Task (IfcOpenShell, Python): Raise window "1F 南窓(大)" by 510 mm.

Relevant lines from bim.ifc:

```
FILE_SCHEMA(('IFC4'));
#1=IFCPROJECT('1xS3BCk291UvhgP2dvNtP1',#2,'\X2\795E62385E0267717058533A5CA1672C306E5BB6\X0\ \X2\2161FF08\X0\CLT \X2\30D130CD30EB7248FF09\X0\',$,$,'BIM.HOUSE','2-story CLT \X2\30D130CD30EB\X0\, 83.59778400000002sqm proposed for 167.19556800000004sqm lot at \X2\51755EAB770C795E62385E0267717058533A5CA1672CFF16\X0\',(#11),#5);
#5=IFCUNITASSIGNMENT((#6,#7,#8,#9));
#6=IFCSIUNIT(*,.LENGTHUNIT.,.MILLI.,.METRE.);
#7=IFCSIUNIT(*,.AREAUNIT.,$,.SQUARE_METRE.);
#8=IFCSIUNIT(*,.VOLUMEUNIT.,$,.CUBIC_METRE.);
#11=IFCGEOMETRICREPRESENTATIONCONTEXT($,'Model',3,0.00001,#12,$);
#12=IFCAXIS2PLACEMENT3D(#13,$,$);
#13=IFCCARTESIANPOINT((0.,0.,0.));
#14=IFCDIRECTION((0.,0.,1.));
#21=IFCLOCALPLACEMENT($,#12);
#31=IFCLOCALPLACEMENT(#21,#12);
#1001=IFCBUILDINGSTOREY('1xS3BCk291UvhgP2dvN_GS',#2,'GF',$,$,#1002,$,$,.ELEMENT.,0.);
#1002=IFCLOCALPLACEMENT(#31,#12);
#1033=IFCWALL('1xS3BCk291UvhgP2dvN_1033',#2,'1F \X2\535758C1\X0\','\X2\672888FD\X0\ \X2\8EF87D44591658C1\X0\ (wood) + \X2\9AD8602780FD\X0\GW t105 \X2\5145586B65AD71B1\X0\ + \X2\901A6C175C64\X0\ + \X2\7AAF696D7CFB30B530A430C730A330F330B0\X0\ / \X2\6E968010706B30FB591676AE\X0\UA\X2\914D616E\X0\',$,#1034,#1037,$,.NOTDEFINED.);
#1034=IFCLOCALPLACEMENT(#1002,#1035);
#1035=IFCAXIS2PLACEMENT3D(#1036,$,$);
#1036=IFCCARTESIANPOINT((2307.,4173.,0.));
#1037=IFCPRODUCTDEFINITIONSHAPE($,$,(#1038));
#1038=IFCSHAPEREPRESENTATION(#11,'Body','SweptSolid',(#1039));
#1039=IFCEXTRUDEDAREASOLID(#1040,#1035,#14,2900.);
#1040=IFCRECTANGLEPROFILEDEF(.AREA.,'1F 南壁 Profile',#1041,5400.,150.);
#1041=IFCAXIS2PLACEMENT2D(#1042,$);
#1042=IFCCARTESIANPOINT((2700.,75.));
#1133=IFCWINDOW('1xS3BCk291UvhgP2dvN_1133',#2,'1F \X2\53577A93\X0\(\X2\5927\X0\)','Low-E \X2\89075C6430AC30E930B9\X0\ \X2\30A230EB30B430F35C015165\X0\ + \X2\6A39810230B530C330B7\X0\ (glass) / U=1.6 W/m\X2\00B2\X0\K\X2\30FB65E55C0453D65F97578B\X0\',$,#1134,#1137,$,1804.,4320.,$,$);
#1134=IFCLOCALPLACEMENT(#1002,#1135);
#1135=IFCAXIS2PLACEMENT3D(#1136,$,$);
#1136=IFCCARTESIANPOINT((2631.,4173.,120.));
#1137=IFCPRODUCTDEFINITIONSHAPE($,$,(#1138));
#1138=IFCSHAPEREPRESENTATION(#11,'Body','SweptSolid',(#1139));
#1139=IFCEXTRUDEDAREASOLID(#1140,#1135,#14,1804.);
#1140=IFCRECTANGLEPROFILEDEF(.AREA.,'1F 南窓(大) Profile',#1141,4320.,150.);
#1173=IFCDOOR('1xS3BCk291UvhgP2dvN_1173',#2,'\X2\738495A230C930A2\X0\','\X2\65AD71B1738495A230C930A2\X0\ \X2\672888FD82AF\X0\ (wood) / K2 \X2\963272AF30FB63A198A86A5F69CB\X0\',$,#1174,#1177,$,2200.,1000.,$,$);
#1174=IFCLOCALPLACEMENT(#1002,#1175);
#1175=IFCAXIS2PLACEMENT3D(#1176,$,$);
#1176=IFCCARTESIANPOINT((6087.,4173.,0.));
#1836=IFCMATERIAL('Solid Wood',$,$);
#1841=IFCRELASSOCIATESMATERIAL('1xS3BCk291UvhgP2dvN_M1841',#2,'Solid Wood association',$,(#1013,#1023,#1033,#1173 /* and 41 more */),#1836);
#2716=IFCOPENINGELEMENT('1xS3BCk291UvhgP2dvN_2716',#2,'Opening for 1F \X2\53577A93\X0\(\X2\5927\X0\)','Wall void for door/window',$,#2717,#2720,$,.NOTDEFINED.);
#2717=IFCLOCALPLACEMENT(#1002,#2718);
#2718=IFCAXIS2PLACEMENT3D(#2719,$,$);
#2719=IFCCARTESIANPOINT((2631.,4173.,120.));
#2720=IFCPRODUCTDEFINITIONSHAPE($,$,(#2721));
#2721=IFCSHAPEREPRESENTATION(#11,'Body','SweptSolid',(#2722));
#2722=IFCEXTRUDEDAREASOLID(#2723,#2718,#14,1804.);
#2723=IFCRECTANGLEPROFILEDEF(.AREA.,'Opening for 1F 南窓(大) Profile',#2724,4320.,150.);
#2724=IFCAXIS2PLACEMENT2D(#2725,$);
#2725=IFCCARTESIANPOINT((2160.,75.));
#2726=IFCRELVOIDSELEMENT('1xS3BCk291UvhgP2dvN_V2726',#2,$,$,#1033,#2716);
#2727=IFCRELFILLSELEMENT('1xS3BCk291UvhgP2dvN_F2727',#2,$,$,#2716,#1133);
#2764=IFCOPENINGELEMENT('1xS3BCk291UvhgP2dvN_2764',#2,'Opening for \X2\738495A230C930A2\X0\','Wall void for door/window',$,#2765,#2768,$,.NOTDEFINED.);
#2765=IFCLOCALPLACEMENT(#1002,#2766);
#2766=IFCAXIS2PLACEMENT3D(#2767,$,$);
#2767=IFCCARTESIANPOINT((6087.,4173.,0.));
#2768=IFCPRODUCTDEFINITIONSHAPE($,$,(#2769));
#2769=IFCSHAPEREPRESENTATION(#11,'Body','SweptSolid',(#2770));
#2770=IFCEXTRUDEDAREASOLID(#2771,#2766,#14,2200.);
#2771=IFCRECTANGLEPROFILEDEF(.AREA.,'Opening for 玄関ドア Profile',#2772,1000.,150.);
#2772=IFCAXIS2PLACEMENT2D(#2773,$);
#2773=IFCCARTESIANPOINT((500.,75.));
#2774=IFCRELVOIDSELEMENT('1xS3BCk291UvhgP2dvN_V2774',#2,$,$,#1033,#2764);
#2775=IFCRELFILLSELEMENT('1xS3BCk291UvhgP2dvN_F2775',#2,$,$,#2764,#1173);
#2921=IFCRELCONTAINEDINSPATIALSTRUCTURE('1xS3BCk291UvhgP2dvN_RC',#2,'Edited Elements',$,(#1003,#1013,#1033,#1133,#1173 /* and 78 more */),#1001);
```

```python
import numpy as np
import ifcopenshell
import ifcopenshell.api.geometry
import ifcopenshell.util.placement
import ifcopenshell.util.unit

model = ifcopenshell.open("bim.ifc")
unit_scale = ifcopenshell.util.unit.calculate_unit_scale(model)

window = model.by_id(1133)
opening = window.FillsVoids[0].RelatingOpeningElement
dz = 0.51 / unit_scale

shift = np.array([0.0, 0.0, dz])
# The window is not placed relative to its opening, so move both.
for product in (opening, window):
    matrix = ifcopenshell.util.placement.get_local_placement(product.ObjectPlacement)
    matrix[:3, 3] += shift
    ifcopenshell.api.geometry.edit_object_placement(model, product=product, matrix=matrix, is_si=False)

print(f"moved by {dz * unit_scale:+.3f} m")

model.write("bim-out.ifc")
```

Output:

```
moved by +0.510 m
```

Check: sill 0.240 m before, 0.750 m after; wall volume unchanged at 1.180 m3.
